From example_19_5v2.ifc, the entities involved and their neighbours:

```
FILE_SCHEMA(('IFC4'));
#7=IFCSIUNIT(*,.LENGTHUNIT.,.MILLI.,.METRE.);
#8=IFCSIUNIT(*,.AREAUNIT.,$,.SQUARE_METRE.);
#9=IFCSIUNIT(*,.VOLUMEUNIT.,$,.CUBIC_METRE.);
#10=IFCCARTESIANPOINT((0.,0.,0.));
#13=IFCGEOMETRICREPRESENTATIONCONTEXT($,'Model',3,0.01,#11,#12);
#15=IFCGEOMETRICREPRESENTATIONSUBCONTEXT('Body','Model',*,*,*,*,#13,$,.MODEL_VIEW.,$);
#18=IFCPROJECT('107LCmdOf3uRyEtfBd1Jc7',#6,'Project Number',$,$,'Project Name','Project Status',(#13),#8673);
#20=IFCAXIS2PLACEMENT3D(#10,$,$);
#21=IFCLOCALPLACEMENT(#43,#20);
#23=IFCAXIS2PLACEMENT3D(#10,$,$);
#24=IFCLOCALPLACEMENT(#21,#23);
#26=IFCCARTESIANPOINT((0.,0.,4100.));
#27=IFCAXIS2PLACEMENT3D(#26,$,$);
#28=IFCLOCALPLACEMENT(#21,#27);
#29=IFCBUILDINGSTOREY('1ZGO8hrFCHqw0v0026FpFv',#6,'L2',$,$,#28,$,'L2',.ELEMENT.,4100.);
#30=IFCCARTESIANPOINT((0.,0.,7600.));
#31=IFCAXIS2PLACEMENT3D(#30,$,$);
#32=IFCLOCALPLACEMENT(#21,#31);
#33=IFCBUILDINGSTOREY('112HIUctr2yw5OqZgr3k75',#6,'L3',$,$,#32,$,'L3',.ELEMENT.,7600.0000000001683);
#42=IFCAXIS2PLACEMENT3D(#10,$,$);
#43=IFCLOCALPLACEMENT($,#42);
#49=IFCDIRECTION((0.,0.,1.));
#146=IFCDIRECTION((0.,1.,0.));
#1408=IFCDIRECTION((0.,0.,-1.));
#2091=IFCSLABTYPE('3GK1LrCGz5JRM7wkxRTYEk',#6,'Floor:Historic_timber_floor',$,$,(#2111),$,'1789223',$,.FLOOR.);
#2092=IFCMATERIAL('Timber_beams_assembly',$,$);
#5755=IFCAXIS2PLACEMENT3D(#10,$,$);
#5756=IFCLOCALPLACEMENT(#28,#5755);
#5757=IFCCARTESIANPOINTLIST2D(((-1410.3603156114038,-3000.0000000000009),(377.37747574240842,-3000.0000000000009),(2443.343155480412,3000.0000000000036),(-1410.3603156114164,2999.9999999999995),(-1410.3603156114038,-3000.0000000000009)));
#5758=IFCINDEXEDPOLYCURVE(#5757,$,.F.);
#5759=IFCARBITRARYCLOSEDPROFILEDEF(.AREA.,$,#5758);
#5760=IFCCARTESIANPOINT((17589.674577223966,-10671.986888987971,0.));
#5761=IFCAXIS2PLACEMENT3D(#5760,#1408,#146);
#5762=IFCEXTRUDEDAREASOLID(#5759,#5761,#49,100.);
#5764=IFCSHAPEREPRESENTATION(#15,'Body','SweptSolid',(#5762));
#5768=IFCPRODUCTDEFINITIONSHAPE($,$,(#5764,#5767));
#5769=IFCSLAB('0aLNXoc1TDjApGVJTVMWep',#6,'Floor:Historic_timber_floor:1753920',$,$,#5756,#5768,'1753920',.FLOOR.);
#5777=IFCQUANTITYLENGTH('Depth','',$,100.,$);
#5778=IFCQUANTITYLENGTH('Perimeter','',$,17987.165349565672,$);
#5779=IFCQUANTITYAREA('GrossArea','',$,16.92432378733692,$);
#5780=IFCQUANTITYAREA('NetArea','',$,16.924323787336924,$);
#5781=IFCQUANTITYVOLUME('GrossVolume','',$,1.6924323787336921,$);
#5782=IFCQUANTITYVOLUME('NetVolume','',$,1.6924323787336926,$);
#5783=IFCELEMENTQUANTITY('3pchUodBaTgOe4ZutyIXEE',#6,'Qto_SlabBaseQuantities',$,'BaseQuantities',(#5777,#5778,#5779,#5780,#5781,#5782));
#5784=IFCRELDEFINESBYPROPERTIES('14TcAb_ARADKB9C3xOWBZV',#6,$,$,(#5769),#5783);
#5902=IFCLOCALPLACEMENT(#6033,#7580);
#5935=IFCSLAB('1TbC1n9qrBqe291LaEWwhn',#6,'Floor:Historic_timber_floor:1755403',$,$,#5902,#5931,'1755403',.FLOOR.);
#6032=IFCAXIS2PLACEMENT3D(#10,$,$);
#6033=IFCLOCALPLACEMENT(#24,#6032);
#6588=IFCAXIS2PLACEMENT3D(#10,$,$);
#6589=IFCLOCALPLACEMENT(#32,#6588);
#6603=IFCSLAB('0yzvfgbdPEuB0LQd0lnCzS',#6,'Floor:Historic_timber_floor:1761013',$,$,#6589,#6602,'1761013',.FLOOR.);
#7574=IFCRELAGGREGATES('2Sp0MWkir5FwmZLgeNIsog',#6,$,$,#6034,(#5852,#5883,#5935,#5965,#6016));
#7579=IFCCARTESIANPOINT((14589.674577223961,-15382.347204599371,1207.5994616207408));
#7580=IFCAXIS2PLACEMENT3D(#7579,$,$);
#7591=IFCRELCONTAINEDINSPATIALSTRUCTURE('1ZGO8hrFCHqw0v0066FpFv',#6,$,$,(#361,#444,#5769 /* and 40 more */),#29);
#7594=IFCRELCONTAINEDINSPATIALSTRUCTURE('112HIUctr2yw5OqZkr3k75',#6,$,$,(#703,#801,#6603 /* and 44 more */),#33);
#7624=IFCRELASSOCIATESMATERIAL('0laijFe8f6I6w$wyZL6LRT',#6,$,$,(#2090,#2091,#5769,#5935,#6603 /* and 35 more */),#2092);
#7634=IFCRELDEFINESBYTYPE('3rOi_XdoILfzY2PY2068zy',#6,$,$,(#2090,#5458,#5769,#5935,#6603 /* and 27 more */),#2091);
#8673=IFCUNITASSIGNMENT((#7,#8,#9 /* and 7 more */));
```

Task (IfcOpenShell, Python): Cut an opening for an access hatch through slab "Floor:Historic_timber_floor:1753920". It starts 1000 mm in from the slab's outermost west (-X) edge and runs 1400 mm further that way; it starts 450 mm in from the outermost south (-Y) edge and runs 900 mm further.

```python
import numpy as np
import ifcopenshell
import ifcopenshell.api.feature
import ifcopenshell.api.geometry
import ifcopenshell.api.pset
import ifcopenshell.api.root
import ifcopenshell.geom
import ifcopenshell.util.element
import ifcopenshell.util.placement
import ifcopenshell.util.representation
import ifcopenshell.util.shape
import ifcopenshell.util.unit

model = ifcopenshell.open("example_19_5v2.ifc")
unit_scale = ifcopenshell.util.unit.calculate_unit_scale(model)
area_scale = ifcopenshell.util.unit.calculate_unit_scale(model, "AREAUNIT")
volume_scale = ifcopenshell.util.unit.calculate_unit_scale(model, "VOLUMEUNIT")
settings = ifcopenshell.geom.settings()


def volume(element):
    """Net volume in cubic metres, openings subtracted."""
    shape = ifcopenshell.geom.create_shape(settings, element)
    return ifcopenshell.util.shape.get_volume(shape.geometry)


slab = model.by_id(5769)
before = volume(slab)

# Extent in the slab's own axes, in metres. The edges named are its -X and -Y sides.
slab_shape = ifcopenshell.geom.create_shape(settings, slab)
vertices = ifcopenshell.util.shape.get_vertices(slab_shape.geometry)
x_min, y_min, bottom = vertices.min(axis=0)
top = vertices[:, 2].max()

opening = ifcopenshell.api.root.create_entity(model, ifc_class="IfcOpeningElement", name="Access hatch opening", predefined_type="OPENING")
context = ifcopenshell.util.representation.get_context(model, "Model", "Body", "MODEL_VIEW")
width, depth = 1.4, 0.9
outline = [(0.0, 0.0), (width, 0.0), (width, depth), (0.0, depth), (0.0, 0.0)]
# Overshoot both faces by 50 mm so the cut is clean.
shape = ifcopenshell.api.geometry.add_slab_representation(
    model, context=context, depth=top - bottom + 0.1, polyline=outline
)
ifcopenshell.api.geometry.assign_representation(model, product=opening, representation=shape)

matrix = ifcopenshell.util.placement.get_local_placement(slab.ObjectPlacement)
matrix[:, 3] = matrix @ np.append(np.array([x_min + 1, y_min + 0.45, bottom - 0.05]) / unit_scale, 1.0)
ifcopenshell.api.geometry.edit_object_placement(model, product=opening, matrix=matrix, is_si=False)
ifcopenshell.api.feature.add_feature(model, feature=opening, element=slab)

after = volume(slab)

# Update the slab's stored quantities.
qto = model.by_id(ifcopenshell.util.element.get_pset(slab, "Qto_SlabBaseQuantities", should_inherit=False)["id"])
ifcopenshell.api.pset.edit_qto(model, qto=qto, properties={
    "NetArea": after / (top - bottom) / area_scale,
    "NetVolume": after / volume_scale,
})

print(f"slab volume {before:.3f} -> {after:.3f} m3")

model.write("example_19_5v2-out.ifc")
```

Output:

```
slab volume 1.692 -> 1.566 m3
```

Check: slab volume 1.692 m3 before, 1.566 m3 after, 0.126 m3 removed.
